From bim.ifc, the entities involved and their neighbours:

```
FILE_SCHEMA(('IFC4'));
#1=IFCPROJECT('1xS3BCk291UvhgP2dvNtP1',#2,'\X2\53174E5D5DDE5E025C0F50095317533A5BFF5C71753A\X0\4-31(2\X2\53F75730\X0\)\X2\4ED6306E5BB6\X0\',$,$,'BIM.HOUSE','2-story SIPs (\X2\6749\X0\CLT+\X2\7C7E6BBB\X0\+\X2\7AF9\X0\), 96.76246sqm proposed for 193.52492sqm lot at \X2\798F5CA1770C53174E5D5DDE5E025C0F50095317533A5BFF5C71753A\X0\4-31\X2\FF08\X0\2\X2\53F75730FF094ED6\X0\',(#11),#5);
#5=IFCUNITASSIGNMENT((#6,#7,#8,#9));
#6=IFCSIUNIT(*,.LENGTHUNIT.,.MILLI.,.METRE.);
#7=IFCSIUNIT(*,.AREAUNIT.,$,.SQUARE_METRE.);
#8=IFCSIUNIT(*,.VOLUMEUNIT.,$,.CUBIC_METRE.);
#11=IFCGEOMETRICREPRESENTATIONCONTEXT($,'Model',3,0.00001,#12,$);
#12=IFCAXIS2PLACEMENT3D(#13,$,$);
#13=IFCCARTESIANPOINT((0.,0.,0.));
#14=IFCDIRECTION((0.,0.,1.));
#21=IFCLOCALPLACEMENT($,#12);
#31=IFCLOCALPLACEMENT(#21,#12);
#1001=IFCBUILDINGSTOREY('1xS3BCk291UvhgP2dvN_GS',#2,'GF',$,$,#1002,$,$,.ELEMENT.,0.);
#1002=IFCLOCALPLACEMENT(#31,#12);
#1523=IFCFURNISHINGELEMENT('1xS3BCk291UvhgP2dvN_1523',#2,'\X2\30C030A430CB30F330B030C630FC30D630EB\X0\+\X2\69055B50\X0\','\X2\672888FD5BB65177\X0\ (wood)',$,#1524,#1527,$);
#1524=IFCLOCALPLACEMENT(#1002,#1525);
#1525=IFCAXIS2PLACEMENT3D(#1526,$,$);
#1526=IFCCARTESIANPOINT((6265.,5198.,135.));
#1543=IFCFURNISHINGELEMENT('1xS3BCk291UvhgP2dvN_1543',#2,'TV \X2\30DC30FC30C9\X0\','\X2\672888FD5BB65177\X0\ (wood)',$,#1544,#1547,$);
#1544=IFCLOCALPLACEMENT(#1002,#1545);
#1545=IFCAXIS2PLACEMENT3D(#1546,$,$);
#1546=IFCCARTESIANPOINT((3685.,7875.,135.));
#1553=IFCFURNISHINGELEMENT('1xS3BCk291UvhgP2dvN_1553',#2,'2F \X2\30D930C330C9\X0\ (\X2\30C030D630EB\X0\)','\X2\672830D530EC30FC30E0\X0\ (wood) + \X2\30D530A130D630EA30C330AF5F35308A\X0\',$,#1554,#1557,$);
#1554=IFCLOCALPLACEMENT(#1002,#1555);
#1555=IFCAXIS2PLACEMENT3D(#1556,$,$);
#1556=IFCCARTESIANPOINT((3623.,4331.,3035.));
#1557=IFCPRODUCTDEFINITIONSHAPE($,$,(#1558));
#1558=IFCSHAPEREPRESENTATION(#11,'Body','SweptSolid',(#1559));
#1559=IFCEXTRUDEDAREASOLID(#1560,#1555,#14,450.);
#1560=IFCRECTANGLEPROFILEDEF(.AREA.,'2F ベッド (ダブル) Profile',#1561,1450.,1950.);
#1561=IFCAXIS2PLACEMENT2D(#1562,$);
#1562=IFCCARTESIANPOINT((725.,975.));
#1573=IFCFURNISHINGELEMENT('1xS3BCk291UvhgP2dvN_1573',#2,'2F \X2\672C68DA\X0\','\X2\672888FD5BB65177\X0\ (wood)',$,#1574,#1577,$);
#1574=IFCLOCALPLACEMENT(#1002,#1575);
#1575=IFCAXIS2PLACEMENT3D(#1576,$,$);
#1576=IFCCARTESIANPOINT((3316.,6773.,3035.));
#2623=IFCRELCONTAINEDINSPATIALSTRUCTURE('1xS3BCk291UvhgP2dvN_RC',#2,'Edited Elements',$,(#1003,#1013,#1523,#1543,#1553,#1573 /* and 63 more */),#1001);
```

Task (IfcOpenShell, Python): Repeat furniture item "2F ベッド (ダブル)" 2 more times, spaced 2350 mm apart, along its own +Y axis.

```python
import ifcopenshell
import ifcopenshell.api.geometry
import ifcopenshell.api.root
import ifcopenshell.util.element
import ifcopenshell.util.placement
import ifcopenshell.util.unit

model = ifcopenshell.open("bim.ifc")
unit_scale = ifcopenshell.util.unit.calculate_unit_scale(model)


def reuse_history(source, copy):
    """copy_class also copies each property set's owner history, people and application; keep the originals."""
    for rel in copy.IsDefinedBy:
        if rel.is_a("IfcRelDefinesByProperties") and (history := rel.RelatingPropertyDefinition.OwnerHistory):
            rel.RelatingPropertyDefinition.OwnerHistory = source.OwnerHistory
            ifcopenshell.util.element.remove_deep2(model, history)


source = model.by_id(1553)
base = ifcopenshell.util.placement.get_local_placement(source.ObjectPlacement)
step = base[:3, 1] * 2.35 / unit_scale

for i in range(1, 3):
    copy = ifcopenshell.api.root.copy_class(model, product=source)
    copy.Representation = ifcopenshell.util.element.copy_deep(
        model, source.Representation, exclude=["IfcGeometricRepresentationContext", "IfcRepresentationMap"]
    )
    reuse_history(source, copy)
    matrix = base.copy()
    matrix[:3, 3] += i * step
    print("added at", matrix[:3, 3].round(3) + 0.0)
    ifcopenshell.api.geometry.edit_object_placement(model, product=copy, matrix=matrix, is_si=False)

model.write("bim_updated.ifc")
```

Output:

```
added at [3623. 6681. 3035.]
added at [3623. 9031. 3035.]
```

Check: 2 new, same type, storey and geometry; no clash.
